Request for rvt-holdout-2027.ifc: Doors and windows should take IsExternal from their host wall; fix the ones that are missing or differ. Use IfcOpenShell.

First a look at what the model holds.

```python
import ifcopenshell
import ifcopenshell.util.element

model = ifcopenshell.open("rvt-holdout-2027.ifc")
print(model.schema)
seen = {}
for e in model.by_type("IfcDoor") + model.by_type("IfcWindow"):
    if not e.FillsVoids:
        continue
    host = e.FillsVoids[0].RelatingOpeningElement.VoidsElements[0].RelatingBuildingElement
    own = ifcopenshell.util.element.get_pset(e, f"Pset_{e.is_a()[3:].removesuffix('StandardCase')}Common", "IsExternal")
    wall = ifcopenshell.util.element.get_pset(host, "Pset_WallCommon", "IsExternal")
    seen[e.is_a(), own, wall] = seen.get((e.is_a(), own, wall), 0) + 1
for (cls, own, wall), count in sorted(seen.items(), key=str):
    print(count, cls, "IsExternal:", own, "| host wall:", wall)
```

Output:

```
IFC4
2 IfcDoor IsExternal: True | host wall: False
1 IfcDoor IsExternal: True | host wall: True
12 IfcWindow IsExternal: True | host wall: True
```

```python
import ifcopenshell
import ifcopenshell.api.pset
import ifcopenshell.util.element

model = ifcopenshell.open("rvt-holdout-2027.ifc")

count = 0
for ifc_class, pset_name in (("IfcDoor", "Pset_DoorCommon"), ("IfcWindow", "Pset_WindowCommon")):
    for e in model.by_type(ifc_class):
        if not e.FillsVoids:
            continue
        host = e.FillsVoids[0].RelatingOpeningElement.VoidsElements[0].RelatingBuildingElement
        external = ifcopenshell.util.element.get_pset(host, "Pset_WallCommon", "IsExternal")
        if external is None or ifcopenshell.util.element.get_pset(e, pset_name, "IsExternal") == external:
            continue
        pset = ifcopenshell.api.pset.add_pset(model, product=e, name=pset_name)
        ifcopenshell.api.pset.edit_pset(model, pset=pset, properties={"IsExternal": external})
        count += 1

print(count, "updated")

model.write("rvt-holdout-2027_v2.ifc")
```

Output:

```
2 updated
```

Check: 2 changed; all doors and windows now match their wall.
